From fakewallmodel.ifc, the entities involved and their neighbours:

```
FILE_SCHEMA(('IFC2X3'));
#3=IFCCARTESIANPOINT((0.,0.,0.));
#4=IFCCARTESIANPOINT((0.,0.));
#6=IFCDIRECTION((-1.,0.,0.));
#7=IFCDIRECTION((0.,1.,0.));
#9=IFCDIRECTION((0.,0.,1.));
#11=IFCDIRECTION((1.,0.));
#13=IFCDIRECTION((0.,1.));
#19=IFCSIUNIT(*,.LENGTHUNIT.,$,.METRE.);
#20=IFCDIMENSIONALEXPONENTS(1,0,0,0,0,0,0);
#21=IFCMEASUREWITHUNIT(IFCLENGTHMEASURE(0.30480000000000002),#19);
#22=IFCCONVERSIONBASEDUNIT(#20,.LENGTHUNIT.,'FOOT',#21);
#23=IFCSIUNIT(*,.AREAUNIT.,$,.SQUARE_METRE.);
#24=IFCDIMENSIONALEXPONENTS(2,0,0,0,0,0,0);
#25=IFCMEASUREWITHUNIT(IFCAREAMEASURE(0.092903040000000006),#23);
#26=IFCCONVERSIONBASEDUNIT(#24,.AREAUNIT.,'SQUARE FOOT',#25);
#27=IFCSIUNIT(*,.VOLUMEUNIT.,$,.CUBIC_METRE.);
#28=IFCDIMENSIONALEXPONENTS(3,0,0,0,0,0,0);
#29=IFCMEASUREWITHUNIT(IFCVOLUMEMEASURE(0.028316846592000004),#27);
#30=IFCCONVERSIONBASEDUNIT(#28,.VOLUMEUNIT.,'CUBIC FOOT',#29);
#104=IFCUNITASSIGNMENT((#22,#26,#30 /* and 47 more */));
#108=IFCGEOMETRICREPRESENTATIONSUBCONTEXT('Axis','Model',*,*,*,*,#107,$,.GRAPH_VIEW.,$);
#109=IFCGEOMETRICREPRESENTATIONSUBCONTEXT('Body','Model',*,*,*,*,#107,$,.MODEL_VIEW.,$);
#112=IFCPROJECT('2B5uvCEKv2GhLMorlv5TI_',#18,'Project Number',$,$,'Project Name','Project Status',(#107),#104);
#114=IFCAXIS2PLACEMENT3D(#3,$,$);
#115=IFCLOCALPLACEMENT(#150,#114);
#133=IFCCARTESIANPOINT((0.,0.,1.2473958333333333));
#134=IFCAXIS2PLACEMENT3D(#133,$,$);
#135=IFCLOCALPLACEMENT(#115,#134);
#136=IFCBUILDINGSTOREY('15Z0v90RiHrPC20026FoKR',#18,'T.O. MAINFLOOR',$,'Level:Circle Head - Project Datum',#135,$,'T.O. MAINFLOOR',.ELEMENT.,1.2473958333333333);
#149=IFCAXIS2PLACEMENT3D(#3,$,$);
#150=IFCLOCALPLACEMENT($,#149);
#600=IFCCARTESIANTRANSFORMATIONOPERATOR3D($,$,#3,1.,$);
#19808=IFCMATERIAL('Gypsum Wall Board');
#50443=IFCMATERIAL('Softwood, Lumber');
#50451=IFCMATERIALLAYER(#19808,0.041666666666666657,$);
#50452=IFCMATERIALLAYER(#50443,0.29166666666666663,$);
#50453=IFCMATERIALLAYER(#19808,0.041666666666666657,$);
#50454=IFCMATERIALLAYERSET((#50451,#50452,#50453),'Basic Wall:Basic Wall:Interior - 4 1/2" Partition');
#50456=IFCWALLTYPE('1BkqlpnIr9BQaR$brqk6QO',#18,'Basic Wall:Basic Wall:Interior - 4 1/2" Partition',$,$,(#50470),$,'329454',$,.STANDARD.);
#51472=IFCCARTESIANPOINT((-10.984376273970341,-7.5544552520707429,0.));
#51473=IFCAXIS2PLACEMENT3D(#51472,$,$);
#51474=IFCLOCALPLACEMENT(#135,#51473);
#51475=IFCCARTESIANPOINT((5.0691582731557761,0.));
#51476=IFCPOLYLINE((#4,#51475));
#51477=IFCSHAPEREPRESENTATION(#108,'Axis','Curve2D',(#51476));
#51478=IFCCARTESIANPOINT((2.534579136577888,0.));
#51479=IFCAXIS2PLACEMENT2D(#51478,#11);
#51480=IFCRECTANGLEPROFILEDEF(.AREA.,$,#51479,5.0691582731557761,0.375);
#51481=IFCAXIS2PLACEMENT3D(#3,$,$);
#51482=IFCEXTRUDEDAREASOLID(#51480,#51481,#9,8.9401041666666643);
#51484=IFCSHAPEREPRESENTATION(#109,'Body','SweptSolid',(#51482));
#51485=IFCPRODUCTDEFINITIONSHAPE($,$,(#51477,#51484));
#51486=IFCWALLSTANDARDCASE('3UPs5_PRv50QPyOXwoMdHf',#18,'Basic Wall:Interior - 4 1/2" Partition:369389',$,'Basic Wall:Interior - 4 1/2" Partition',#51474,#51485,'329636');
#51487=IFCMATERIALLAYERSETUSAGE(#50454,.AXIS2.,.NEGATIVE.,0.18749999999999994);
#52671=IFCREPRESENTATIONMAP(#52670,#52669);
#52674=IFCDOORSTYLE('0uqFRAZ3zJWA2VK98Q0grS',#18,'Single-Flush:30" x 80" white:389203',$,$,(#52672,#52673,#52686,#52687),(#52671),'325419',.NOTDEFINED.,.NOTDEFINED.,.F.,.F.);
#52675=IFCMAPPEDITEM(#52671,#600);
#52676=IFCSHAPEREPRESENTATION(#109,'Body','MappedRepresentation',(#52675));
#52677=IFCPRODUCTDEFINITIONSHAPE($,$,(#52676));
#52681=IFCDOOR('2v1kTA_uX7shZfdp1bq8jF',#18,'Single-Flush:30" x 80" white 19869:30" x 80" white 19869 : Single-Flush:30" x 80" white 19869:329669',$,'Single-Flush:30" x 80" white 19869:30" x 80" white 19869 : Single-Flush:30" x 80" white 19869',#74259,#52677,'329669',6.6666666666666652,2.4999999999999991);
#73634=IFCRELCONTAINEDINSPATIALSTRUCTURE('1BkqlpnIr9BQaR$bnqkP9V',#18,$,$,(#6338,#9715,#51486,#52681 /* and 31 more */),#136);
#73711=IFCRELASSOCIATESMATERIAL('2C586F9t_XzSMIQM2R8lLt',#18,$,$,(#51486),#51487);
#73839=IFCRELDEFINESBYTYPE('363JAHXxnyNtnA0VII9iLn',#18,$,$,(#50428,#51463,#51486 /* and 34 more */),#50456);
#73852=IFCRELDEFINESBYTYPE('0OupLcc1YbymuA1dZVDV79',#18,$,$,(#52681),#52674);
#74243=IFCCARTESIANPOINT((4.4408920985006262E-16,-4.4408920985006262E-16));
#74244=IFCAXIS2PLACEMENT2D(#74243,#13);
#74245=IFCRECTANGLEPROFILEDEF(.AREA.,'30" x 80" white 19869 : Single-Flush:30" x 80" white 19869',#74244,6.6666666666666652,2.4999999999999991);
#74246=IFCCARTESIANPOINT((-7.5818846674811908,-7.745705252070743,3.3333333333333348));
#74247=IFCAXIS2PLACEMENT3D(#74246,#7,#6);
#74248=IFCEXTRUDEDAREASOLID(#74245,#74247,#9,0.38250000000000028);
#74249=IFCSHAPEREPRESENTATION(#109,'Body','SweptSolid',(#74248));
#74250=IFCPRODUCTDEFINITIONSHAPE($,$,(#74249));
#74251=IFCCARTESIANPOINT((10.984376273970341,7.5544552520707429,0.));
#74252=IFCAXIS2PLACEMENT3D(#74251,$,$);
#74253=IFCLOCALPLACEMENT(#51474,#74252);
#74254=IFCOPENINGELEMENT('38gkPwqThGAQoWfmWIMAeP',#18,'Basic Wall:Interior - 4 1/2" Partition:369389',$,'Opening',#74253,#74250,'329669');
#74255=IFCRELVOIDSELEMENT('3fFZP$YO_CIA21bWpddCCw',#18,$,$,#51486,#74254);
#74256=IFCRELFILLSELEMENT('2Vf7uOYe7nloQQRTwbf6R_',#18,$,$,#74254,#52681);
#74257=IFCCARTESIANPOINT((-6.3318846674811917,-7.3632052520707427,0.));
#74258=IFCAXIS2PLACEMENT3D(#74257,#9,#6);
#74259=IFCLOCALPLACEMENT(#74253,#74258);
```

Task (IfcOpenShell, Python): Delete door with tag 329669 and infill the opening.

```python
import ifcopenshell
import ifcopenshell.api.feature
import ifcopenshell.api.root
import ifcopenshell.geom
import ifcopenshell.util.shape

model = ifcopenshell.open("fakewallmodel.ifc")
settings = ifcopenshell.geom.settings()


def volume(element):
    """Net volume in cubic metres, openings subtracted."""
    shape = ifcopenshell.geom.create_shape(settings, element)
    return ifcopenshell.util.shape.get_volume(shape.geometry)


door = model.by_guid("2v1kTA_uX7shZfdp1bq8jF")
opening = door.FillsVoids[0].RelatingOpeningElement
wall = opening.VoidsElements[0].RelatingBuildingElement
before = volume(wall)

ifcopenshell.api.root.remove_product(model, product=door)
ifcopenshell.api.feature.remove_feature(model, feature=opening)

after = volume(wall)

print(f"wall volume {before:.3f} -> {after:.3f} m3")

model.write("fakewallmodel_v2.ifc")
```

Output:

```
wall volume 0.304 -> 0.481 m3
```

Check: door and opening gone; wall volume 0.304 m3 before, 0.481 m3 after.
